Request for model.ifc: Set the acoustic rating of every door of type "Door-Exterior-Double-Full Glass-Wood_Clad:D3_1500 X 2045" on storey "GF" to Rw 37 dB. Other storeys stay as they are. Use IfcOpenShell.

First a look at what the model holds.

```python
import ifcopenshell
import ifcopenshell.util.element

model = ifcopenshell.open("model.ifc")
print(model.schema)
storey = next(s for s in model.by_type("IfcBuildingStorey") if s.Name == "GF")
doors = [e for e in ifcopenshell.util.element.get_decomposition(storey) if e.is_a("IfcDoor")]
seen = {}
for e in doors:
    element_type = ifcopenshell.util.element.get_type(e)
    key = (element_type.Name if element_type != e and element_type else None, ifcopenshell.util.element.get_pset(e, "Pset_DoorCommon", "AcousticRating"))
    seen[key] = seen.get(key, 0) + 1
for (name, value), count in sorted(seen.items(), key=str):
    print(count, "x", name, "|", value)
```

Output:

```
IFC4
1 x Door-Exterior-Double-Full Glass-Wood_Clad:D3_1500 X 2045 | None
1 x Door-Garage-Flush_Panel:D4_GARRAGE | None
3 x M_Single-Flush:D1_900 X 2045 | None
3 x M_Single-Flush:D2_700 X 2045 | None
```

```python
import ifcopenshell
import ifcopenshell.api.pset
import ifcopenshell.util.element

model = ifcopenshell.open("model.ifc")

storey = next(s for s in model.by_type("IfcBuildingStorey") if s.Name == "GF")
doors = [e for e in ifcopenshell.util.element.get_decomposition(storey) if e.is_a("IfcDoor")]

count = 0
for e in doors:
    element_type = ifcopenshell.util.element.get_type(e)
    if element_type in (None, e) or element_type.Name != "Door-Exterior-Double-Full Glass-Wood_Clad:D3_1500 X 2045":
        continue
    # add_pset returns the element's existing set when there is one.
    pset = ifcopenshell.api.pset.add_pset(model, product=e, name="Pset_DoorCommon")
    ifcopenshell.api.pset.edit_pset(model, pset=pset, properties={"AcousticRating": "Rw 37 dB"})
    count += 1

print(count, "doors updated")

model.write("model_updated.ifc")
```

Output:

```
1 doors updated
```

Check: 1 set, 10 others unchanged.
